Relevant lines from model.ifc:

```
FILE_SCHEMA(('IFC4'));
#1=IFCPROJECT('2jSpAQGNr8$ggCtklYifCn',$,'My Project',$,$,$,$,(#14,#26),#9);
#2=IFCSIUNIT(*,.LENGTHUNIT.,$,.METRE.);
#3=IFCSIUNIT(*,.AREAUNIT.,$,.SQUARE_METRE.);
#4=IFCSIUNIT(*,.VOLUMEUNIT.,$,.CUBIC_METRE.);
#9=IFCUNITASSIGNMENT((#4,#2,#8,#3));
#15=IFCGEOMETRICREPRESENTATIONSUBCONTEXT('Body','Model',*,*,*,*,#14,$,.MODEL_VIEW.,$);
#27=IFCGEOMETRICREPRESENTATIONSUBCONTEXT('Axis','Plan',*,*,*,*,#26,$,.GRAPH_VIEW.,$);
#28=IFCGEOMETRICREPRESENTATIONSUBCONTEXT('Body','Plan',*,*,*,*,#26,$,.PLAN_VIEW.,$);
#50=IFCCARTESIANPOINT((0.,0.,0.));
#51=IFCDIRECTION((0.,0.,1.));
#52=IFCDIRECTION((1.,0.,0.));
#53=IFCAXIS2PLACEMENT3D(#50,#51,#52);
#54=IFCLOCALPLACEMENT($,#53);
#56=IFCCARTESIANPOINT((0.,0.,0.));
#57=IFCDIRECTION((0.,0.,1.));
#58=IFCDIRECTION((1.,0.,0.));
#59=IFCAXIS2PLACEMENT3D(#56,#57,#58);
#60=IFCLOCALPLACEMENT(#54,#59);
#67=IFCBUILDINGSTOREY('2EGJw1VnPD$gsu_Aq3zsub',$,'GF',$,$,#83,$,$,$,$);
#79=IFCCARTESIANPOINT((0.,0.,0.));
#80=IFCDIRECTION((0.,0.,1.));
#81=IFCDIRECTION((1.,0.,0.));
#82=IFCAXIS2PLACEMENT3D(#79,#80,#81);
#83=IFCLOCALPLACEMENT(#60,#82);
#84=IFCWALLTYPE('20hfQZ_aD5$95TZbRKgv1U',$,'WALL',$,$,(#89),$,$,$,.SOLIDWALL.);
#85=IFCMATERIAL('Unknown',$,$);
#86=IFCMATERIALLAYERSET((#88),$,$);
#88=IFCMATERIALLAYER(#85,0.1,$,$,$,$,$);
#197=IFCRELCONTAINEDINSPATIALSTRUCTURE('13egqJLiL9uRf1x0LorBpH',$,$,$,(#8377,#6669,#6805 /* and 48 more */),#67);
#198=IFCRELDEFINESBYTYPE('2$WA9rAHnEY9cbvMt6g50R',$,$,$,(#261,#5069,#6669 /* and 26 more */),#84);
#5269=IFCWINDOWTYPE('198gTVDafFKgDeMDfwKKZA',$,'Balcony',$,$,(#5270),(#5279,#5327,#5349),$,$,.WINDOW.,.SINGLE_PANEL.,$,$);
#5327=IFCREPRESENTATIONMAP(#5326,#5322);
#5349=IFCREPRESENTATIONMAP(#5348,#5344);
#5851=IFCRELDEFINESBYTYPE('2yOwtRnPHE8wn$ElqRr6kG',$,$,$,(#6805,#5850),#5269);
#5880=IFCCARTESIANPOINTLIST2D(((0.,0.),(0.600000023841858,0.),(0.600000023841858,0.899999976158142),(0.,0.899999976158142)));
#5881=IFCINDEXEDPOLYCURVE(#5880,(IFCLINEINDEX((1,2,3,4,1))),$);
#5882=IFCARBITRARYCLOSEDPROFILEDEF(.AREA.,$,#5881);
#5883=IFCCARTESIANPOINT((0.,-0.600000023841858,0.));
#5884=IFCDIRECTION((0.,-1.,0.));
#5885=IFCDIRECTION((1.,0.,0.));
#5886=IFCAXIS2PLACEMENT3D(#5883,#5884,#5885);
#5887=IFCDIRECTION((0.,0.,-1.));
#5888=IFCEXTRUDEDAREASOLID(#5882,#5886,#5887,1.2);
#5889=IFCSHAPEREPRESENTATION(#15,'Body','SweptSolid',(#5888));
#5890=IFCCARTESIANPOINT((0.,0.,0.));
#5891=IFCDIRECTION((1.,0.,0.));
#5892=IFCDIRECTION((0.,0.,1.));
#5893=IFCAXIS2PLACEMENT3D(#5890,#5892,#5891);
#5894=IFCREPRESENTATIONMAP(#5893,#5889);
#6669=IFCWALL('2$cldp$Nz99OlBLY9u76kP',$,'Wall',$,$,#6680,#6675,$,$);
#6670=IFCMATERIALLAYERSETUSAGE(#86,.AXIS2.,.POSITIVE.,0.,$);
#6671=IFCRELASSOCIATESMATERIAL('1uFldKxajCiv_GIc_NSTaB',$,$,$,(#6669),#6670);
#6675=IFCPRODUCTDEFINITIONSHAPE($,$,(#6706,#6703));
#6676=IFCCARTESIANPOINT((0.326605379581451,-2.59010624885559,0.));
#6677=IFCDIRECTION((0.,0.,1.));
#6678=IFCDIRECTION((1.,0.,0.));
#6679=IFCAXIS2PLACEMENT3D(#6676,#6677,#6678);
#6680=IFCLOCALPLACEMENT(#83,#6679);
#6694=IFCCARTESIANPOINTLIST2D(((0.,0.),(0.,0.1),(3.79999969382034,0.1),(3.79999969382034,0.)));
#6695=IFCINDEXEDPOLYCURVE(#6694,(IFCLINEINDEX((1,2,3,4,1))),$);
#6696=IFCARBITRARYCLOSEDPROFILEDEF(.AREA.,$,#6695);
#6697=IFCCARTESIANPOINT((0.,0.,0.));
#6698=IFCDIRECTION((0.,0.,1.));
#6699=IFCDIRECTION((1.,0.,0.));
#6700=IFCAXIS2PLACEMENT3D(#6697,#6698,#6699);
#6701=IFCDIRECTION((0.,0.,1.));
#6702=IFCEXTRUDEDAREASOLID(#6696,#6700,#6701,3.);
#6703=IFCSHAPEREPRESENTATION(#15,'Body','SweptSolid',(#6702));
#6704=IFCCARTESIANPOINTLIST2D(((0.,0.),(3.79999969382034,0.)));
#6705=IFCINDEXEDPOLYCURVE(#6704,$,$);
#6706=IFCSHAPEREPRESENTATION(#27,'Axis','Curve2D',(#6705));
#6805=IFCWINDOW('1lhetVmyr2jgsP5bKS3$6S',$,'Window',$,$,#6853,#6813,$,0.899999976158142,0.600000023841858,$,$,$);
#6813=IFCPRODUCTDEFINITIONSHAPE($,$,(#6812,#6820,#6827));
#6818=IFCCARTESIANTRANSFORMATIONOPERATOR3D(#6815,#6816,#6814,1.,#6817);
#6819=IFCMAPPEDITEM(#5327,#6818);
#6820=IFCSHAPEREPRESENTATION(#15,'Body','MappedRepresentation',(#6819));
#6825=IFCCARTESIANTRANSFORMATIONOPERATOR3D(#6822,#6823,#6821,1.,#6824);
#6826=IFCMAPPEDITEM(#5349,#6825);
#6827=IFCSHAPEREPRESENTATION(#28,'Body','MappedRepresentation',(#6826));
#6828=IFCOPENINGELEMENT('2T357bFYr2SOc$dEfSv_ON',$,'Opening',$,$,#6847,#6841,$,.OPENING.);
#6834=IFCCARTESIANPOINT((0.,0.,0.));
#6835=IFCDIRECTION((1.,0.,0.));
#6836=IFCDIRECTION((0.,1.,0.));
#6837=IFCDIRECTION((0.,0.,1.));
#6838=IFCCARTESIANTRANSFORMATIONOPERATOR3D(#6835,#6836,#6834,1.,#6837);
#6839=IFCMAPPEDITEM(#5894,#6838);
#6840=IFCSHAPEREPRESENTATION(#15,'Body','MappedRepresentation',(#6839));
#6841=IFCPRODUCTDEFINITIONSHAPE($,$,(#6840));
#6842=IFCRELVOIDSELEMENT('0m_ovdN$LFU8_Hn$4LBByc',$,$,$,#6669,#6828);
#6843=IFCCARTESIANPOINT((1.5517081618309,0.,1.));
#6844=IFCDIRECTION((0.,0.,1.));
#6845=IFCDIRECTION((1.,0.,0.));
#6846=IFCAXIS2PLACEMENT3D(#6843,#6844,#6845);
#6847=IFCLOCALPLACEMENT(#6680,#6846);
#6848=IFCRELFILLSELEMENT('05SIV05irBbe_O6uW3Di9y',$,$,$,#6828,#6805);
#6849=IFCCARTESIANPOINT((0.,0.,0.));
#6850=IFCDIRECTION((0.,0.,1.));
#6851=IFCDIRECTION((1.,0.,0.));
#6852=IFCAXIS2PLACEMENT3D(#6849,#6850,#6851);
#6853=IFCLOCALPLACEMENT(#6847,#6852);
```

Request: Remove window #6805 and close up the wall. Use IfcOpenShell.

```python
import ifcopenshell
import ifcopenshell.api.feature
import ifcopenshell.api.root
import ifcopenshell.geom
import ifcopenshell.util.shape

model = ifcopenshell.open("model.ifc")
settings = ifcopenshell.geom.settings()


def volume(element):
    """Net volume in cubic metres, openings subtracted."""
    shape = ifcopenshell.geom.create_shape(settings, element)
    return ifcopenshell.util.shape.get_volume(shape.geometry)


window = model.by_guid("1lhetVmyr2jgsP5bKS3$6S")
opening = window.FillsVoids[0].RelatingOpeningElement
wall = opening.VoidsElements[0].RelatingBuildingElement
before = volume(wall)

ifcopenshell.api.root.remove_product(model, product=window)
ifcopenshell.api.feature.remove_feature(model, feature=opening)

after = volume(wall)

print(f"wall volume {before:.3f} -> {after:.3f} m3")

model.write("model-out.ifc")
```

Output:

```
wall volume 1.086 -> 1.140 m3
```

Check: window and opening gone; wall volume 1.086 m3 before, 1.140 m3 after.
